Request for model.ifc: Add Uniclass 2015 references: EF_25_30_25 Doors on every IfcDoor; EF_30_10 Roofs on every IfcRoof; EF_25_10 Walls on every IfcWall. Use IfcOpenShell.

First a look at what the model holds.

```python
import ifcopenshell

model = ifcopenshell.open("model.ifc")
print(model.schema)
print("classifications:", [c.Name for c in model.by_type("IfcClassification")])
for ifc_class in ("IfcDoor", "IfcRoof", "IfcStair", "IfcWall", "IfcWindow"):
    print(ifc_class, len(model.by_type(ifc_class)))
```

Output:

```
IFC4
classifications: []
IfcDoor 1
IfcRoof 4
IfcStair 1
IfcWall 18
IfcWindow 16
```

```python
import ifcopenshell
import ifcopenshell.api.classification

model = ifcopenshell.open("model.ifc")

system = ifcopenshell.api.classification.add_classification(model, classification="Uniclass 2015")

codes = {
    "IfcDoor": ("EF_25_30_25", "Doors"),
    "IfcRoof": ("EF_30_10", "Roofs"),
    "IfcWall": ("EF_25_10", "Walls"),
}
for ifc_class, (code, name) in codes.items():
    products = model.by_type(ifc_class)
    ifcopenshell.api.classification.add_reference(
        model, products=products, classification=system, identification=code, name=name
    )
    print(code, len(products))

model.write("model_rev.ifc")
```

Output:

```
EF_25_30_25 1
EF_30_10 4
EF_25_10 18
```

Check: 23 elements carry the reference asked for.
